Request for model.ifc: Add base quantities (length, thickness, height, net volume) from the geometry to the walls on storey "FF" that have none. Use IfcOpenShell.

First a look at what the model holds.

```python
import ifcopenshell
import ifcopenshell.util.element
import ifcopenshell.util.unit

model = ifcopenshell.open("model.ifc")
print(model.schema)
for unit_type in ("LENGTHUNIT", "AREAUNIT", "VOLUMEUNIT"):
    print(unit_type, ifcopenshell.util.unit.calculate_unit_scale(model, unit_type))
storey = next(s for s in model.by_type("IfcBuildingStorey") if s.Name == "FF")
walls = [e for e in ifcopenshell.util.element.get_decomposition(storey) if e.is_a("IfcWall")]
for e in sorted(walls, key=lambda e: e.id()):
    print(e.id(), e.is_a(), e.Name, list(ifcopenshell.util.element.get_psets(e, qtos_only=True)), sep=" | ")
```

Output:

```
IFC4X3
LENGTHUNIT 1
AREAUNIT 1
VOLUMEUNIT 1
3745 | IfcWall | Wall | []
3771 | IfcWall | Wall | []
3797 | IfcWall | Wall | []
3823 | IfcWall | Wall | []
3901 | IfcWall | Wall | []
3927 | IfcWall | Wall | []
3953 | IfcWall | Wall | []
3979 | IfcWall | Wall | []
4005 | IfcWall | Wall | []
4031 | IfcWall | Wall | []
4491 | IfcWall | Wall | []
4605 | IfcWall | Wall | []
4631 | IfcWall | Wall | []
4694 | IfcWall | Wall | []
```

```python
import ifcopenshell
import ifcopenshell.api.pset
import ifcopenshell.geom
import ifcopenshell.util.element
import ifcopenshell.util.shape
import ifcopenshell.util.unit

model = ifcopenshell.open("model.ifc")
unit_scale = ifcopenshell.util.unit.calculate_unit_scale(model)
volume_scale = ifcopenshell.util.unit.calculate_unit_scale(model, "VOLUMEUNIT")
settings = ifcopenshell.geom.settings()

storey = next(s for s in model.by_type("IfcBuildingStorey") if s.Name == "FF")
walls = [e for e in ifcopenshell.util.element.get_decomposition(storey) if e.is_a("IfcWall")]

for e in sorted(walls, key=lambda e: e.id()):
    if ifcopenshell.util.element.get_psets(e, qtos_only=True, should_inherit=False):
        continue
    # Geometry comes back in metres, in the element's own axes.
    shape = ifcopenshell.geom.create_shape(settings, e)
    values = {
        "Length": ifcopenshell.util.shape.get_x(shape.geometry) / unit_scale,
        "Width": ifcopenshell.util.shape.get_y(shape.geometry) / unit_scale,
        "Height": ifcopenshell.util.shape.get_z(shape.geometry) / unit_scale,
        "NetVolume": ifcopenshell.util.shape.get_volume(shape.geometry) / volume_scale,
    }
    qto = ifcopenshell.api.pset.add_qto(model, product=e, name="Qto_WallBaseQuantities")
    ifcopenshell.api.pset.edit_qto(model, qto=qto, properties=values)
    print(e.id(), {k: round(v, 3) for k, v in values.items()})

model.write("model_v2.ifc")
```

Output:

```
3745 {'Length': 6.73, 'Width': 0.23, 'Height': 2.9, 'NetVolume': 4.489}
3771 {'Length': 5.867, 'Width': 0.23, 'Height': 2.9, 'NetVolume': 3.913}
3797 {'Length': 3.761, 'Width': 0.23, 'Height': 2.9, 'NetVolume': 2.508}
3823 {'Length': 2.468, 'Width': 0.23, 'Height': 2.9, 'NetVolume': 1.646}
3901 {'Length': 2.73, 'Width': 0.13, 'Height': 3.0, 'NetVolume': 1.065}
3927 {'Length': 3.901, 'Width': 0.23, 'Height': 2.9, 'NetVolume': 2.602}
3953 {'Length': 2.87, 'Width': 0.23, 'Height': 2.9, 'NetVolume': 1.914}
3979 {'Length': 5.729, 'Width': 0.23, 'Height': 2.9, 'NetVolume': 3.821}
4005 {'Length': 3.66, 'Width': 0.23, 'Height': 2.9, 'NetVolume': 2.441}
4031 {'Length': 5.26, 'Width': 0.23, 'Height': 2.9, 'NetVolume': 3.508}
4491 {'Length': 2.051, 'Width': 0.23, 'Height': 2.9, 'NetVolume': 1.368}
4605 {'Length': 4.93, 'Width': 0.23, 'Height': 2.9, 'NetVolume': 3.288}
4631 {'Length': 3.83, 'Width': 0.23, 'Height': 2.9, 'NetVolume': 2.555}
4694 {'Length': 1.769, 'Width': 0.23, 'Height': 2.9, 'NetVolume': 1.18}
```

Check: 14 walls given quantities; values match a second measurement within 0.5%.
